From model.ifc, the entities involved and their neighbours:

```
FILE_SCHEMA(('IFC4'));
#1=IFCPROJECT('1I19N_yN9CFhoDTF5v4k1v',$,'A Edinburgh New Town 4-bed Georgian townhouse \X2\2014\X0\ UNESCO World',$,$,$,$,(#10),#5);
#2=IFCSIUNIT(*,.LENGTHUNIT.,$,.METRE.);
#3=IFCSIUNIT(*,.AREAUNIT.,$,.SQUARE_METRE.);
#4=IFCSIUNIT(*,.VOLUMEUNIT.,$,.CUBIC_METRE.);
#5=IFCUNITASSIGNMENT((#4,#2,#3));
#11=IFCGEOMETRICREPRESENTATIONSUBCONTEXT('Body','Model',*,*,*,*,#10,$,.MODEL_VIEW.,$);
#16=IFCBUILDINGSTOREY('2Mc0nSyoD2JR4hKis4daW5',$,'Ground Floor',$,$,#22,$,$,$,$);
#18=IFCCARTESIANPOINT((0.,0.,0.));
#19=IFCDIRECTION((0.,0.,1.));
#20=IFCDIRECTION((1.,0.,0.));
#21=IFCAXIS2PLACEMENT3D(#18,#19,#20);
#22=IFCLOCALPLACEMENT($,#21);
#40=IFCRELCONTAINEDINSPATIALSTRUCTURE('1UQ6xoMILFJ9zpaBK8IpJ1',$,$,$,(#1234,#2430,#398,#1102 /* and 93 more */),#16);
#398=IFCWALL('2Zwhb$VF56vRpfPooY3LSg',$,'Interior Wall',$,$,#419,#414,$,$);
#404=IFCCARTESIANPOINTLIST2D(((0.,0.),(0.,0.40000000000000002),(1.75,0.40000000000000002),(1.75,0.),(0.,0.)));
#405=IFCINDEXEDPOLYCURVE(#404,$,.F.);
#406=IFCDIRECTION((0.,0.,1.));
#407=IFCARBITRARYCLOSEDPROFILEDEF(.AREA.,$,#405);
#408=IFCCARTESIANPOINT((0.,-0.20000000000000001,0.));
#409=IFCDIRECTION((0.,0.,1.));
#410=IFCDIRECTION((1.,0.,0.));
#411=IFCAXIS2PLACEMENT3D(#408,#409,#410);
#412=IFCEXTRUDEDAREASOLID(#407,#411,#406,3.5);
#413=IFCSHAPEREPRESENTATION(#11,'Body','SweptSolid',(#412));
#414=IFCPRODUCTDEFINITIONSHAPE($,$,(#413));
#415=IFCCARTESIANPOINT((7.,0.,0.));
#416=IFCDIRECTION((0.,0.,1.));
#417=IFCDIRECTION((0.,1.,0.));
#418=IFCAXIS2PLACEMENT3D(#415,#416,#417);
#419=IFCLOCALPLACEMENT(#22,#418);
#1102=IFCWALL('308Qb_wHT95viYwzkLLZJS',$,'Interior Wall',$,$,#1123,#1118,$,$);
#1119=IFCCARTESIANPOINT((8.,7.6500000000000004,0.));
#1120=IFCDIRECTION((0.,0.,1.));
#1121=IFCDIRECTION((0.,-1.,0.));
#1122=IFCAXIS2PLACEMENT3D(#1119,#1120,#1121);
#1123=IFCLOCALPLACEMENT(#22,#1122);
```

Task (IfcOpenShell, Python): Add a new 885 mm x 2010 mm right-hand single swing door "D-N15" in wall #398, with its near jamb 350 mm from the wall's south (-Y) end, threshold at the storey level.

```python
import numpy as np
import ifcopenshell
import ifcopenshell.api.feature
import ifcopenshell.api.geometry
import ifcopenshell.api.root
import ifcopenshell.api.spatial
import ifcopenshell.geom
import ifcopenshell.util.element
import ifcopenshell.util.placement
import ifcopenshell.util.representation
import ifcopenshell.util.shape
import ifcopenshell.util.unit

model = ifcopenshell.open("model.ifc")
unit_scale = ifcopenshell.util.unit.calculate_unit_scale(model)
settings = ifcopenshell.geom.settings()


def volume(element):
    """Net volume in cubic metres, openings subtracted."""
    shape = ifcopenshell.geom.create_shape(settings, element)
    return ifcopenshell.util.shape.get_volume(shape.geometry)


wall = model.by_guid("2Zwhb$VF56vRpfPooY3LSg")
storey = ifcopenshell.util.element.get_container(wall, ifc_class="IfcBuildingStorey")
context = ifcopenshell.util.representation.get_context(model, "Model", "Body", "MODEL_VIEW")
before = volume(wall)

width, height, from_end, sill = 0.885, 2.01, 0.35, 0.0  # metres

# The wall runs along its own X axis, and the end named is its -X end.
wall_shape = ifcopenshell.geom.create_shape(settings, wall)
x, y, z = ifcopenshell.util.shape.get_vertices(wall_shape.geometry).T
start = x.min() + from_end
face, thickness = float(y.min()), float(y.max() - y.min())
wall_matrix = ifcopenshell.util.placement.get_local_placement(wall.ObjectPlacement)
level = ifcopenshell.util.placement.get_local_placement(storey.ObjectPlacement)[2, 3]


def in_wall(x, y):
    """Placement at x, y metres in the wall's axes, at sill height."""
    matrix = wall_matrix.copy()
    matrix[:, 3] = wall_matrix @ np.array([x / unit_scale, y / unit_scale, 0.0, 1.0])
    matrix[2, 3] = level + sill / unit_scale
    return matrix


# Opening: a box that overshoots both wall faces by 50 mm.
opening = ifcopenshell.api.root.create_entity(model, ifc_class="IfcOpeningElement", predefined_type="OPENING")
box = ifcopenshell.api.geometry.add_wall_representation(
    model, context=context, length=width, height=height, thickness=thickness + 0.1
)
ifcopenshell.api.geometry.assign_representation(model, product=opening, representation=box)
ifcopenshell.api.geometry.edit_object_placement(model, product=opening, matrix=in_wall(start, face - 0.05), is_si=False)
ifcopenshell.api.feature.add_feature(model, feature=opening, element=wall)

door = ifcopenshell.api.root.create_entity(model, ifc_class="IfcDoor", name="D-N15", predefined_type="DOOR")
door.OverallWidth, door.OverallHeight = width / unit_scale, height / unit_scale
door.OperationType = "SINGLE_SWING_RIGHT"
body = ifcopenshell.api.geometry.add_door_representation(
    model,
    context=context,
    overall_width=door.OverallWidth,
    overall_height=door.OverallHeight,
    operation_type="SINGLE_SWING_RIGHT",
    lining_properties={"LiningDepth": thickness / unit_scale, "ThresholdDepth": thickness / unit_scale},
)
ifcopenshell.api.geometry.assign_representation(model, product=door, representation=body)
ifcopenshell.api.spatial.assign_container(model, products=[door], relating_structure=storey)
ifcopenshell.api.feature.add_filling(model, opening=opening, element=door)

# The lining spans the wall, so the door starts at the wall face.
ifcopenshell.api.geometry.edit_object_placement(model, product=door, matrix=in_wall(start, face), is_si=False)

after = volume(wall)

print(f"wall volume {before:.3f} -> {after:.3f} m3")

model.write("model_updated.ifc")
```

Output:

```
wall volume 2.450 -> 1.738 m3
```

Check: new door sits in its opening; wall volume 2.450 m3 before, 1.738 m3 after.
